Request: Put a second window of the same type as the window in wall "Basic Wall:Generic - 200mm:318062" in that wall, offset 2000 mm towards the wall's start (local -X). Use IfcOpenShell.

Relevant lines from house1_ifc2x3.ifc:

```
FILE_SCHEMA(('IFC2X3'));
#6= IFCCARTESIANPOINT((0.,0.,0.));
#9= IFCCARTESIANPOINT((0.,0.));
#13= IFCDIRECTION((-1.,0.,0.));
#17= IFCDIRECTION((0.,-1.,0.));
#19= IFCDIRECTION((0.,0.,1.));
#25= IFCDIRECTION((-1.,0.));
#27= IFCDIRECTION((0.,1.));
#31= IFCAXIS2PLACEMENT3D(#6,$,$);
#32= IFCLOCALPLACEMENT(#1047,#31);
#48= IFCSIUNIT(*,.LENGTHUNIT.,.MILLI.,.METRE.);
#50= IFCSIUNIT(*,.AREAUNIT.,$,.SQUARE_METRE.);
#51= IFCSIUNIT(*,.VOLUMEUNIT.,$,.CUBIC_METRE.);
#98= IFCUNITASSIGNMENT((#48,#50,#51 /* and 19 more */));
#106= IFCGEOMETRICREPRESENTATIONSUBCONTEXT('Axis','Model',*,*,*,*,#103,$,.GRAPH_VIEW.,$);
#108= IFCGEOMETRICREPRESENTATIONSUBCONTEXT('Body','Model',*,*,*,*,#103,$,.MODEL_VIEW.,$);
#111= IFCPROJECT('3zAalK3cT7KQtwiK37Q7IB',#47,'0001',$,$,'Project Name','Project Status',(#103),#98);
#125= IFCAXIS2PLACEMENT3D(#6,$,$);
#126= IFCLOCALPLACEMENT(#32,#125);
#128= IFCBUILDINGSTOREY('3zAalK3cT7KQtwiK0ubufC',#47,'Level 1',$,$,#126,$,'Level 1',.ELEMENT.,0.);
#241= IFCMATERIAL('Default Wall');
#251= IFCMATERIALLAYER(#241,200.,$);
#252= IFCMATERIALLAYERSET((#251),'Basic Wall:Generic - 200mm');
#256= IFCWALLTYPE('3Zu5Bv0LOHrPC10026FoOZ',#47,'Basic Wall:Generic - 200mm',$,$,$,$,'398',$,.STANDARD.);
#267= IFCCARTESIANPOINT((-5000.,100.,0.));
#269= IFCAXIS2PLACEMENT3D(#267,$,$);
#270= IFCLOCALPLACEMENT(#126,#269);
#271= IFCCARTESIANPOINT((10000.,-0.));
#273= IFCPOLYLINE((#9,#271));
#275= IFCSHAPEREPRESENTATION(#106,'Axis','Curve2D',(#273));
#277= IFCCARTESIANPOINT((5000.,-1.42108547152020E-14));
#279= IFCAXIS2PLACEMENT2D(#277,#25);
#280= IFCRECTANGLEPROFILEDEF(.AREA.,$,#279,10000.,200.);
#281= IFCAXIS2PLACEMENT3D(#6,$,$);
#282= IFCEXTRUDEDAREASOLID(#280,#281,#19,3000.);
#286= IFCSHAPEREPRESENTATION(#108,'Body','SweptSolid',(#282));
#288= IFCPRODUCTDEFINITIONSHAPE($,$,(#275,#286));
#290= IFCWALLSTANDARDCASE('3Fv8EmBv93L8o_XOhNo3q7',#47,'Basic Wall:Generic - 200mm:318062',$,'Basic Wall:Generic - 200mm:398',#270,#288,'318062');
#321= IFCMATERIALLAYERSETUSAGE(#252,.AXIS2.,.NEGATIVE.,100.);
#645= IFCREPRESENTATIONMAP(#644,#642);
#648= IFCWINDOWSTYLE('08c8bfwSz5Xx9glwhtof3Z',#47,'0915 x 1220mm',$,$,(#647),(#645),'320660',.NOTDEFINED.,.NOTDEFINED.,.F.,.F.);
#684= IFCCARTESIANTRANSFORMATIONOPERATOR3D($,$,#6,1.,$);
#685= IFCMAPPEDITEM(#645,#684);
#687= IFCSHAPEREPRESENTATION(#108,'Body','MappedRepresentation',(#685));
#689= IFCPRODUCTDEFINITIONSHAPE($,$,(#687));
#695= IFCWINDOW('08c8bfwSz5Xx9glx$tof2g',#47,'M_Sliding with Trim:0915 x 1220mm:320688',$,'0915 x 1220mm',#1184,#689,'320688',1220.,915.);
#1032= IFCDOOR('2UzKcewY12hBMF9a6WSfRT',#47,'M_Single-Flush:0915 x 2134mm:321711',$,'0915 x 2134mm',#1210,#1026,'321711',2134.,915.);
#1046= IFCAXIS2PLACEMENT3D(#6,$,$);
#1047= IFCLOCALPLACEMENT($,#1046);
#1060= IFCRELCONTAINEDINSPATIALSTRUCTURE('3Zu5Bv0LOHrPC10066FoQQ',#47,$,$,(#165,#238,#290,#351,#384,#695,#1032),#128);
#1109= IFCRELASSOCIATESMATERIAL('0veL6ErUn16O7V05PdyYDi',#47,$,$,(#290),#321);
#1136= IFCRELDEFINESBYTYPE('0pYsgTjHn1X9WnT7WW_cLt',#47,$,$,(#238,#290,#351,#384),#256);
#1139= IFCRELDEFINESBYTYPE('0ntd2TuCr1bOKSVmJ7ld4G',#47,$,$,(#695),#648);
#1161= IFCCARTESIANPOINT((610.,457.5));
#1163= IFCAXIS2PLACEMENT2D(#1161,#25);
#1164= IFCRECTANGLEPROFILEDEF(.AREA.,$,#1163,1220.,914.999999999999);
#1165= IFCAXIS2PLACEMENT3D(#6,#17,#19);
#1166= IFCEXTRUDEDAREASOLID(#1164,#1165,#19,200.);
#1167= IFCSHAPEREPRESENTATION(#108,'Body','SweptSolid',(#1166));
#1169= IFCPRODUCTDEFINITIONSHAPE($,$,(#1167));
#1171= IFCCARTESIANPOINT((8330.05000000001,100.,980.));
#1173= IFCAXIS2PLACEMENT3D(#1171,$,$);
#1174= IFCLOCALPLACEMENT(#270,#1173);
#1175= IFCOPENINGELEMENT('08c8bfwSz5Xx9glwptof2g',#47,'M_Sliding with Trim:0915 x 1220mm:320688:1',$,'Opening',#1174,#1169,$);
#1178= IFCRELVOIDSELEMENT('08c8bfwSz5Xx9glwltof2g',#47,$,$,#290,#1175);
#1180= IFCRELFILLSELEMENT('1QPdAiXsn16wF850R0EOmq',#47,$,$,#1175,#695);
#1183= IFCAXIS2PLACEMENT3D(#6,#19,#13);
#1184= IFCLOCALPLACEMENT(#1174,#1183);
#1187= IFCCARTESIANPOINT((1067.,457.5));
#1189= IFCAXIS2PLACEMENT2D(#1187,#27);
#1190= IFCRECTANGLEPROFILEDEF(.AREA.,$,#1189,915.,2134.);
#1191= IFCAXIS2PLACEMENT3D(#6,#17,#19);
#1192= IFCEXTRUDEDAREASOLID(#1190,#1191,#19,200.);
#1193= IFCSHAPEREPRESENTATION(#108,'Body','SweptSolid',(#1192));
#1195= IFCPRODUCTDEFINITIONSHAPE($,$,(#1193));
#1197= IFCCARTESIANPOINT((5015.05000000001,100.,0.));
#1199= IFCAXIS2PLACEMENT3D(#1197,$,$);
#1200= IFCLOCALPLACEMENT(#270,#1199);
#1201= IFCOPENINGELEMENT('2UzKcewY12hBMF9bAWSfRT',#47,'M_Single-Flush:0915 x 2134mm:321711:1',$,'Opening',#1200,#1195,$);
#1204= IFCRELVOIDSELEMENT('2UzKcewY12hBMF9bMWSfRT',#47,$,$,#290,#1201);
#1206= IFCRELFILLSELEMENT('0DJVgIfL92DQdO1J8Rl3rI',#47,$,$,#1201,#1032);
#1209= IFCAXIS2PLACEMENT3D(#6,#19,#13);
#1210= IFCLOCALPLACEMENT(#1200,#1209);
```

```python
import ifcopenshell
import ifcopenshell.api.feature
import ifcopenshell.api.geometry
import ifcopenshell.api.root
import ifcopenshell.geom
import ifcopenshell.util.element
import ifcopenshell.util.placement
import ifcopenshell.util.shape
import ifcopenshell.util.unit

model = ifcopenshell.open("house1_ifc2x3.ifc")
unit_scale = ifcopenshell.util.unit.calculate_unit_scale(model)
settings = ifcopenshell.geom.settings()


def volume(element):
    """Net volume in cubic metres, openings subtracted."""
    shape = ifcopenshell.geom.create_shape(settings, element)
    return ifcopenshell.util.shape.get_volume(shape.geometry)


def reuse_history(source, copy):
    """copy_class also copies each property set's owner history, people and application; keep the originals."""
    for rel in copy.IsDefinedBy:
        if rel.is_a("IfcRelDefinesByProperties") and (history := rel.RelatingPropertyDefinition.OwnerHistory):
            rel.RelatingPropertyDefinition.OwnerHistory = source.OwnerHistory
            ifcopenshell.util.element.remove_deep2(model, history)


window = model.by_guid("08c8bfwSz5Xx9glx$tof2g")
opening = window.FillsVoids[0].RelatingOpeningElement
wall = opening.VoidsElements[0].RelatingBuildingElement
before = volume(wall)
shift = ifcopenshell.util.placement.get_local_placement(wall.ObjectPlacement)[:3, 0] * -2 / unit_scale

# copy_class copies the void relationship, type, container and properties, but no geometry.
new_opening = ifcopenshell.api.root.copy_class(model, product=opening)
new_opening.Representation = ifcopenshell.util.element.copy_deep(
    model, opening.Representation, exclude=["IfcGeometricRepresentationContext", "IfcRepresentationMap"]
)
new_opening.Name = "M_Sliding with Trim:0915 x 1220mm"
new_window = ifcopenshell.api.root.copy_class(model, product=window)
new_window.Representation = ifcopenshell.util.element.copy_deep(
    model, window.Representation, exclude=["IfcGeometricRepresentationContext", "IfcRepresentationMap"]
)
new_window.Name = "M_Sliding with Trim:0915 x 1220mm"
new_window.Tag = None
reuse_history(window, new_window)
fills = ifcopenshell.api.feature.add_filling(model, opening=new_opening, element=new_window)
fills.OwnerHistory = new_window.OwnerHistory  # required in IFC2X3

for old, new in ((opening, new_opening), (window, new_window)):
    matrix = ifcopenshell.util.placement.get_local_placement(old.ObjectPlacement)
    matrix[:3, 3] += shift
    ifcopenshell.api.geometry.edit_object_placement(model, product=new, matrix=matrix, is_si=False)

after = volume(wall)

print(f"wall volume {before:.3f} -> {after:.3f} m3")

model.write("house1_ifc2x3-out.ifc")
```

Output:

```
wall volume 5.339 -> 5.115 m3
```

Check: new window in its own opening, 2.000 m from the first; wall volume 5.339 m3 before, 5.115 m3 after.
